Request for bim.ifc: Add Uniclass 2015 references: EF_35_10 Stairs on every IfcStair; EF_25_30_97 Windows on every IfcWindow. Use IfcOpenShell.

First a look at what the model holds.

```python
import ifcopenshell

model = ifcopenshell.open("bim.ifc")
print(model.schema)
print("classifications:", [c.Name for c in model.by_type("IfcClassification")])
for ifc_class in ("IfcDoor", "IfcRoof", "IfcStair", "IfcWall", "IfcWindow"):
    print(ifc_class, len(model.by_type(ifc_class)))
```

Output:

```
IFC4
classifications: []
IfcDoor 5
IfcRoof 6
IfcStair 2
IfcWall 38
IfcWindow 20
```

```python
import ifcopenshell
import ifcopenshell.api.classification

model = ifcopenshell.open("bim.ifc")

system = ifcopenshell.api.classification.add_classification(model, classification="Uniclass 2015")

codes = {
    "IfcStair": ("EF_35_10", "Stairs"),
    "IfcWindow": ("EF_25_30_97", "Windows"),
}
for ifc_class, (code, name) in codes.items():
    products = model.by_type(ifc_class)
    ifcopenshell.api.classification.add_reference(
        model, products=products, classification=system, identification=code, name=name
    )
    print(code, len(products))

model.write("bim_updated.ifc")
```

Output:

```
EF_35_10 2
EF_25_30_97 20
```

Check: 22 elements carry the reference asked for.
